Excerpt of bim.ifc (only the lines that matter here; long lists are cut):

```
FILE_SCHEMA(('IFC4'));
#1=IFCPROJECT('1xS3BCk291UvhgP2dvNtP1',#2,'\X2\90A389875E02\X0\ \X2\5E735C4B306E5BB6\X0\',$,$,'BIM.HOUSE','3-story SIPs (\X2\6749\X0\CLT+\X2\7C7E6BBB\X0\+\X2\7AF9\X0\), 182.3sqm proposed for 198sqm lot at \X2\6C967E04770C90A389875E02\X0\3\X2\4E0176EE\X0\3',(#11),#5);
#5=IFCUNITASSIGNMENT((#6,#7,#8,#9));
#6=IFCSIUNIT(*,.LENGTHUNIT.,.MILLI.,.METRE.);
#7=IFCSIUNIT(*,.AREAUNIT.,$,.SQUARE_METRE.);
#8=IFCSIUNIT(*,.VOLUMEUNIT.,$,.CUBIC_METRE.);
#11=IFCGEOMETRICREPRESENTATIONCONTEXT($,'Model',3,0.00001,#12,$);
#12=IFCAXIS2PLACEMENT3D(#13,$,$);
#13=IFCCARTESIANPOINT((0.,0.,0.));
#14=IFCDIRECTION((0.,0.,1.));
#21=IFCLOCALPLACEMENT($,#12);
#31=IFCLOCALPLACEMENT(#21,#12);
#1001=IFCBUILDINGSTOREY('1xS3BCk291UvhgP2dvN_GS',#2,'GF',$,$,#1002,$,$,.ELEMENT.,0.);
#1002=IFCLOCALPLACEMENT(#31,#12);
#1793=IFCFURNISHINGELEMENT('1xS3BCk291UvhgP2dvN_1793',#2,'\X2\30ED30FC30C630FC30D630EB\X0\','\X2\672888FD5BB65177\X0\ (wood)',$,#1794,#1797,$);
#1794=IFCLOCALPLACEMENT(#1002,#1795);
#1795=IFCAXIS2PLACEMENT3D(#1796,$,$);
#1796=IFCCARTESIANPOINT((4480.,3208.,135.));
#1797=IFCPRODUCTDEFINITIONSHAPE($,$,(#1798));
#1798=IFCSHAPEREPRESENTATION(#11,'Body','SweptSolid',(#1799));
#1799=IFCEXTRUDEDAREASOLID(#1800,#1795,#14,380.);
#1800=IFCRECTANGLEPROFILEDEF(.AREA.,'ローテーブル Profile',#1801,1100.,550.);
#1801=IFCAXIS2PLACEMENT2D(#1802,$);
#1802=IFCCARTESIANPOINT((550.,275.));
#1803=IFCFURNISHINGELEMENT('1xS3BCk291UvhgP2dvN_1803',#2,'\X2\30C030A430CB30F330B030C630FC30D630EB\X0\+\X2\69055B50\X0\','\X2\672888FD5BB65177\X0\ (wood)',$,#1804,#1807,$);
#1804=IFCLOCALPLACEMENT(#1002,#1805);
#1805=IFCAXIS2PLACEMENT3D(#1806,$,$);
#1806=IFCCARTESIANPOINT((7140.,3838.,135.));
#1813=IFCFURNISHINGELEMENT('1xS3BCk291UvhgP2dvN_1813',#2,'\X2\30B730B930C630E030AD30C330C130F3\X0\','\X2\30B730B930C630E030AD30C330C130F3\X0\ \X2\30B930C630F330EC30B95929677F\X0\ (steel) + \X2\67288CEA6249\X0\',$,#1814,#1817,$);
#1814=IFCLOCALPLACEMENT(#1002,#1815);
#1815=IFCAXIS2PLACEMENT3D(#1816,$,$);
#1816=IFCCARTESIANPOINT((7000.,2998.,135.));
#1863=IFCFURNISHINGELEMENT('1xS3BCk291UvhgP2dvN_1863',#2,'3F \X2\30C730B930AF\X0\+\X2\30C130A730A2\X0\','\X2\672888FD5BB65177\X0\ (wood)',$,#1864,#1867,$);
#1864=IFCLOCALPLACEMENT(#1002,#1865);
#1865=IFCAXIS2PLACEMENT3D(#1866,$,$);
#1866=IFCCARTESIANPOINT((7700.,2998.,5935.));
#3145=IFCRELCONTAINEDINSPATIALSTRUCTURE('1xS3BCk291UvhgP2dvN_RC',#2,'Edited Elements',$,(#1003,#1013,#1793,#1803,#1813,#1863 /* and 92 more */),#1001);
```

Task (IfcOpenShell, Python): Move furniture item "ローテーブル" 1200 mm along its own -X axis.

```python
import ifcopenshell
import ifcopenshell.api.geometry
import ifcopenshell.util.placement
import ifcopenshell.util.unit

model = ifcopenshell.open("bim.ifc")
unit_scale = ifcopenshell.util.unit.calculate_unit_scale(model)

item = model.by_guid("1xS3BCk291UvhgP2dvN_1793")
matrix = ifcopenshell.util.placement.get_local_placement(item.ObjectPlacement)
matrix[:3, 3] -= matrix[:3, 0] * 1.2 / unit_scale
ifcopenshell.api.geometry.edit_object_placement(model, product=item, matrix=matrix, is_si=False)

print(ifcopenshell.util.placement.get_local_placement(item.ObjectPlacement).round(3) + 0.0)

model.write("bim-out.ifc")
```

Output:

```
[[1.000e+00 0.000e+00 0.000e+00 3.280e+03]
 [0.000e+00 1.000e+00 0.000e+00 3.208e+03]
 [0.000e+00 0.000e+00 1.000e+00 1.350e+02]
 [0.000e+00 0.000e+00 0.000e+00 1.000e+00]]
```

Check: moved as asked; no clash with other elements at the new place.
